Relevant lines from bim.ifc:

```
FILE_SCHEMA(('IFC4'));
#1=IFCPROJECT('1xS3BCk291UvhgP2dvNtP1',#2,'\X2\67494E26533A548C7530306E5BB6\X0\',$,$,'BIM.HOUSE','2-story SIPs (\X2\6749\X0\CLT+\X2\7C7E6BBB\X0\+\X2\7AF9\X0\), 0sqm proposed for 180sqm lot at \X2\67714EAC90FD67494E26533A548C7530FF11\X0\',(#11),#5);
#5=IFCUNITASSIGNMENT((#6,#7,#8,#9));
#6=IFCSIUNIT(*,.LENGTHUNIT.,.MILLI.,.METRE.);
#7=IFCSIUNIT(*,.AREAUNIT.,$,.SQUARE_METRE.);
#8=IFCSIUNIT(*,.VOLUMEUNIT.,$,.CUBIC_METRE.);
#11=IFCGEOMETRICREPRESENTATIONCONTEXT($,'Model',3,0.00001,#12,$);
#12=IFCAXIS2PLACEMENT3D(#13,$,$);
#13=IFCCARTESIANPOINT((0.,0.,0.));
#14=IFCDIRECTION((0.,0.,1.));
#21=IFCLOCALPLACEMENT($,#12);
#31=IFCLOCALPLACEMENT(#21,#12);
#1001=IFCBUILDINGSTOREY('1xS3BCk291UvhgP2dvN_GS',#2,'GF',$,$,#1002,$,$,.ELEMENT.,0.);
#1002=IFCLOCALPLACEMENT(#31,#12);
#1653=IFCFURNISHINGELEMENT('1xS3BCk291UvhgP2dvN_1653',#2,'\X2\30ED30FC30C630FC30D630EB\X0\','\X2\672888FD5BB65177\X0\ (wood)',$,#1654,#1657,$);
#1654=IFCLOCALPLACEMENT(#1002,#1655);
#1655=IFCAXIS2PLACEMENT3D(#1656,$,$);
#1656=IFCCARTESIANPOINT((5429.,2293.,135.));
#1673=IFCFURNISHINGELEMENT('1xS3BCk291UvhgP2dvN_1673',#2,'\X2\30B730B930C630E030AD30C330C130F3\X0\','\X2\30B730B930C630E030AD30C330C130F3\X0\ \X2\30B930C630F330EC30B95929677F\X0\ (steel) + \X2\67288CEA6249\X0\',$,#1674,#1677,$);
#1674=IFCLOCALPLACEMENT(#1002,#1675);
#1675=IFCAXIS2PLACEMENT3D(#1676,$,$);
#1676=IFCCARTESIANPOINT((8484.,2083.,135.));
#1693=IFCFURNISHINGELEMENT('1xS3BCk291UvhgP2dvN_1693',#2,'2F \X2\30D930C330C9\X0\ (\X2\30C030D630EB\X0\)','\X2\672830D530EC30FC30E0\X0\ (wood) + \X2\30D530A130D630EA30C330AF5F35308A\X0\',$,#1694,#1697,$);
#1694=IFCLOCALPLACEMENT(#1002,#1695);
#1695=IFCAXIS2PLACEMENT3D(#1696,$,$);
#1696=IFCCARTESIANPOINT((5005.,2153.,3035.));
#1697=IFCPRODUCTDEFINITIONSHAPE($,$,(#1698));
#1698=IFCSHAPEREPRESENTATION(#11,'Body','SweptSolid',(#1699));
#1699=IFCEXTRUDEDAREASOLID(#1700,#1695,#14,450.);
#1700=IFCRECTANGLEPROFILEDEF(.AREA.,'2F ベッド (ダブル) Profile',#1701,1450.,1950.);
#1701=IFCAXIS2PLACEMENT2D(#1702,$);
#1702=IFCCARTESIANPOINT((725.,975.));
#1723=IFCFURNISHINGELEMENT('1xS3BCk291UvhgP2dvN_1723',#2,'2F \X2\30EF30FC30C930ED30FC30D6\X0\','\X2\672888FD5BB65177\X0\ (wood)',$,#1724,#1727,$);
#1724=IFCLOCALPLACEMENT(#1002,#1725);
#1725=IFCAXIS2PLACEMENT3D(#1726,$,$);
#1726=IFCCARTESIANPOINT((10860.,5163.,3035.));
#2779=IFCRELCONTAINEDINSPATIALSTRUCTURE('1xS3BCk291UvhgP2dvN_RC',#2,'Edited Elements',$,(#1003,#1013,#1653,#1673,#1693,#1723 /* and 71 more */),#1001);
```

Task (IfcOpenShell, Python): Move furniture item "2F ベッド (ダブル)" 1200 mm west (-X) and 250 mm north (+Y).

```python
import ifcopenshell
import ifcopenshell.api.geometry
import ifcopenshell.util.placement
import ifcopenshell.util.unit

model = ifcopenshell.open("bim.ifc")
unit_scale = ifcopenshell.util.unit.calculate_unit_scale(model)

item = model.by_guid("1xS3BCk291UvhgP2dvN_1693")
matrix = ifcopenshell.util.placement.get_local_placement(item.ObjectPlacement)
matrix[0, 3] -= 1.2 / unit_scale
matrix[1, 3] += 0.25 / unit_scale
ifcopenshell.api.geometry.edit_object_placement(model, product=item, matrix=matrix, is_si=False)

print(ifcopenshell.util.placement.get_local_placement(item.ObjectPlacement).round(3) + 0.0)

model.write("bim-out.ifc")
```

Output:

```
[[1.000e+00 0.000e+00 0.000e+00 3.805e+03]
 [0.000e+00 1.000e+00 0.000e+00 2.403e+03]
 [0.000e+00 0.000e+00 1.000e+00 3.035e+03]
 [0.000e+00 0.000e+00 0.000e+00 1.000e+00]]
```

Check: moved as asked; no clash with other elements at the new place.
